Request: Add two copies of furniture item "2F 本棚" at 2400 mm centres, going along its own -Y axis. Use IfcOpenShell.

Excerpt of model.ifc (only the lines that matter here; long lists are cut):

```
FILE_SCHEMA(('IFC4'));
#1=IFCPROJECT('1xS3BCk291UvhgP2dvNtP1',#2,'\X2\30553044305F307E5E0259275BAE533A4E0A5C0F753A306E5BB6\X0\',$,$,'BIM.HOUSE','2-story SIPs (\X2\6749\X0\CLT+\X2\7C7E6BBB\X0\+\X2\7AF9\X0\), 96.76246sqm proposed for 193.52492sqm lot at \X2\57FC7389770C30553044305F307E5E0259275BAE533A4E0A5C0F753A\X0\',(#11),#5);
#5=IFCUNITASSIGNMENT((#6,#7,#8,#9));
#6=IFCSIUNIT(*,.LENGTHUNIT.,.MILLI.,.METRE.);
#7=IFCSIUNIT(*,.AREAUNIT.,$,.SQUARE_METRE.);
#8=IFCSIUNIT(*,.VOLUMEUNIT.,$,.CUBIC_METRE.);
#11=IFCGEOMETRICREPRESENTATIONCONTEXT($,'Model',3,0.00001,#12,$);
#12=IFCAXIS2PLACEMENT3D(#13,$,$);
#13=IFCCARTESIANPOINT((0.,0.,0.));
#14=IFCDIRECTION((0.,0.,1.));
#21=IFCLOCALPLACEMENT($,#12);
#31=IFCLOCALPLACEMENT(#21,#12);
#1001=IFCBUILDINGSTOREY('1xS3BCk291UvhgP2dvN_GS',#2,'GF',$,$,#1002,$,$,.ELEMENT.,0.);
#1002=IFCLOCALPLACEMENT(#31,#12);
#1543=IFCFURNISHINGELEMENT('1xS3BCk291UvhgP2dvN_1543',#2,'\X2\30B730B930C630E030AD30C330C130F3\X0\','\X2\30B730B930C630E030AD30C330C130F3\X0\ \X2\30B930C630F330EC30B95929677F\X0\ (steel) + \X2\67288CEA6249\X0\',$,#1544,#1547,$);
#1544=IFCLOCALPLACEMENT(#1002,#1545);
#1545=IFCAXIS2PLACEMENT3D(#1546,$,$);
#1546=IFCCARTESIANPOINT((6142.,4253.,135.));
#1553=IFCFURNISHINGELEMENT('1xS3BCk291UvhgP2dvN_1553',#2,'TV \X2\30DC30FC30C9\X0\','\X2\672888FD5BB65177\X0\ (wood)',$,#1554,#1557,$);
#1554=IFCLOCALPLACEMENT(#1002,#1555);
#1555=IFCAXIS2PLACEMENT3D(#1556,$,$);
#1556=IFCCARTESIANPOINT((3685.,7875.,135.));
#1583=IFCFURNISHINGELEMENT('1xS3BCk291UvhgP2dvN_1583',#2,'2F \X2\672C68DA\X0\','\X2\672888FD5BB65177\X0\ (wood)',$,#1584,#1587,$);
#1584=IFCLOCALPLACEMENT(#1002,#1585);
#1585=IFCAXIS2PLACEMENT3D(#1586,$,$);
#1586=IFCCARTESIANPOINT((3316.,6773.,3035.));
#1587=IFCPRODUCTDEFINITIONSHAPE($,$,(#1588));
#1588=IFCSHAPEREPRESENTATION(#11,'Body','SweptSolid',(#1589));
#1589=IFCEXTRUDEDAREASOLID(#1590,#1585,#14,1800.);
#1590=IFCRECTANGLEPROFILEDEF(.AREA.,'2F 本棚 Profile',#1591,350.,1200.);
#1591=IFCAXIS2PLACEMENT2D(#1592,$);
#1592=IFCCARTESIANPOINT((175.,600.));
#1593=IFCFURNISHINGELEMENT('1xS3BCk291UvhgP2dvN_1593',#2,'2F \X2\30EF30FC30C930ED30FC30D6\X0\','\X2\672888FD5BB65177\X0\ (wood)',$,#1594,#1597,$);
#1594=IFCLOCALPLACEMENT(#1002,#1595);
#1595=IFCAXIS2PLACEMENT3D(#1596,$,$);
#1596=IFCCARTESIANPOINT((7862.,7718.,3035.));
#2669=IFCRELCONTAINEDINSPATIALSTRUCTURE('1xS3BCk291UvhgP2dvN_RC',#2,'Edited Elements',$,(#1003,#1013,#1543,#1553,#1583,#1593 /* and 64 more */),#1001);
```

```python
import ifcopenshell
import ifcopenshell.api.geometry
import ifcopenshell.api.root
import ifcopenshell.util.element
import ifcopenshell.util.placement
import ifcopenshell.util.unit

model = ifcopenshell.open("model.ifc")
unit_scale = ifcopenshell.util.unit.calculate_unit_scale(model)


def reuse_history(source, copy):
    """copy_class also copies each property set's owner history, people and application; keep the originals."""
    for rel in copy.IsDefinedBy:
        if rel.is_a("IfcRelDefinesByProperties") and (history := rel.RelatingPropertyDefinition.OwnerHistory):
            rel.RelatingPropertyDefinition.OwnerHistory = source.OwnerHistory
            ifcopenshell.util.element.remove_deep2(model, history)


source = model.by_id(1583)
base = ifcopenshell.util.placement.get_local_placement(source.ObjectPlacement)
step = -base[:3, 1] * 2.4 / unit_scale

for i in range(1, 3):
    copy = ifcopenshell.api.root.copy_class(model, product=source)
    copy.Representation = ifcopenshell.util.element.copy_deep(
        model, source.Representation, exclude=["IfcGeometricRepresentationContext", "IfcRepresentationMap"]
    )
    reuse_history(source, copy)
    matrix = base.copy()
    matrix[:3, 3] += i * step
    print("added at", matrix[:3, 3].round(3) + 0.0)
    ifcopenshell.api.geometry.edit_object_placement(model, product=copy, matrix=matrix, is_si=False)

model.write("model_updated.ifc")
```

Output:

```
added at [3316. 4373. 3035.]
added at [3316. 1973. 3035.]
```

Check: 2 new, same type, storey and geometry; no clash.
